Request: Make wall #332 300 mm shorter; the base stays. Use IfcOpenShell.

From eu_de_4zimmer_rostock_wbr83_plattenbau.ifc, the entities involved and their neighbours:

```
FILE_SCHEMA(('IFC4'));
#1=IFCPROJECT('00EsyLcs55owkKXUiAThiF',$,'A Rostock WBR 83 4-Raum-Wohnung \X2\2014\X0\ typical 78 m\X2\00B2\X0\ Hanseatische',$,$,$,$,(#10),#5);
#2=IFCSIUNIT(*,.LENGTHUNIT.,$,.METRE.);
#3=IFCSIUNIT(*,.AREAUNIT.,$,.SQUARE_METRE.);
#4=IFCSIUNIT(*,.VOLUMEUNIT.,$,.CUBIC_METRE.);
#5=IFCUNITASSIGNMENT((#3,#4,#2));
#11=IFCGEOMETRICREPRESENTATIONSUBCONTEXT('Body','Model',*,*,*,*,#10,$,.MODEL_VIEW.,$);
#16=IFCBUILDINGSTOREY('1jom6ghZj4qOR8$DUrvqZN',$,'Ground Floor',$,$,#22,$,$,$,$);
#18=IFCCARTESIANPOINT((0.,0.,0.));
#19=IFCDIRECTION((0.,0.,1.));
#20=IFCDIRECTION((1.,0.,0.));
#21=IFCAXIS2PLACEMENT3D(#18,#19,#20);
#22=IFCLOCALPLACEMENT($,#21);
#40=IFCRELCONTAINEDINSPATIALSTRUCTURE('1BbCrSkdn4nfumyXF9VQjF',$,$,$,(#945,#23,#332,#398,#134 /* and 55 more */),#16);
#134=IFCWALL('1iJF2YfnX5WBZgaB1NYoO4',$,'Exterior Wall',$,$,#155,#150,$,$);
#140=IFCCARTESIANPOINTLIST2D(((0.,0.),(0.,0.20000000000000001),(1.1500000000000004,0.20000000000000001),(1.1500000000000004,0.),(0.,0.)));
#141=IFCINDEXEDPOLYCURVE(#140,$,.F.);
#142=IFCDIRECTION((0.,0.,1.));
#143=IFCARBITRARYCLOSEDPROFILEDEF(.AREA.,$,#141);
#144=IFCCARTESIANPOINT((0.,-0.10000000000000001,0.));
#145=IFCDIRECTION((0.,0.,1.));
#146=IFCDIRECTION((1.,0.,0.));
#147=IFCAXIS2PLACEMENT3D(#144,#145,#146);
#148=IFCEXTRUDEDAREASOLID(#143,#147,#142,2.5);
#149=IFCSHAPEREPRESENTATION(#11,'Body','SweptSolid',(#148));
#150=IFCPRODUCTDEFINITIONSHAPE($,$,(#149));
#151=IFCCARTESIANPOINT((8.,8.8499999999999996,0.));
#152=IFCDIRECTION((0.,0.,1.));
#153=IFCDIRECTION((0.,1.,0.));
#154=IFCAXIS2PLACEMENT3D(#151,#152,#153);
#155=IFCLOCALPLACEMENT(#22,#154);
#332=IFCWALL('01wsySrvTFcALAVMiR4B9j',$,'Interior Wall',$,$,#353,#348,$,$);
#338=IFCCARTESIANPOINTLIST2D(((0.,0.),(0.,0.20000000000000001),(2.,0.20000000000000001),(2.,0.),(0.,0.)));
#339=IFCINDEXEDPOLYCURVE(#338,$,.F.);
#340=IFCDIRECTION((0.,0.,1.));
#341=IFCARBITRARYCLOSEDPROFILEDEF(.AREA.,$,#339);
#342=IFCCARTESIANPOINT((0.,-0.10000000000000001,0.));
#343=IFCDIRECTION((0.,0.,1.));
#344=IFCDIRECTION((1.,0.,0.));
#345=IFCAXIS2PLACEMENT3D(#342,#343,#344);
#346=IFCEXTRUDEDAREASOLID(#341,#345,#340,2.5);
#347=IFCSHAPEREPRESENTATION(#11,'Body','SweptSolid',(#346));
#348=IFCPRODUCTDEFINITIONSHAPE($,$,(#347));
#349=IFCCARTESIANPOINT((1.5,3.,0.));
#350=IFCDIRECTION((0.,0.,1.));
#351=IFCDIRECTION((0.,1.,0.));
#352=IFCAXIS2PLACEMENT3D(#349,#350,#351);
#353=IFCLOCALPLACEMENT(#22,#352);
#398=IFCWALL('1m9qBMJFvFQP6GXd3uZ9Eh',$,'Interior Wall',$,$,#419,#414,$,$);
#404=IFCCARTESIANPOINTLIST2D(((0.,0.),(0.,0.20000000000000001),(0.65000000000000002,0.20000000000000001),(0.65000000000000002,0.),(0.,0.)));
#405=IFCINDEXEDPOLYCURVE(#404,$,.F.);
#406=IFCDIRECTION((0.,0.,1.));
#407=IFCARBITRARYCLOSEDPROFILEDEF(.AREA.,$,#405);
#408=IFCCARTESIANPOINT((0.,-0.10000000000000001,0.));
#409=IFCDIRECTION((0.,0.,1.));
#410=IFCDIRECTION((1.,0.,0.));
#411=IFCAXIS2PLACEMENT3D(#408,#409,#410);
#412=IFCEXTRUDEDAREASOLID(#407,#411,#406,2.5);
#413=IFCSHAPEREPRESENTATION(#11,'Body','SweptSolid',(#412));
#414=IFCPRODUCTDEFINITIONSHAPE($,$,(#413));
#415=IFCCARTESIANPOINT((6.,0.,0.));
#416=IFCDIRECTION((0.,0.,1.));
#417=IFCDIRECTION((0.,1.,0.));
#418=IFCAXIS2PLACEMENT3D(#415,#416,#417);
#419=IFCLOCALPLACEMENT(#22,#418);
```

```python
import ifcopenshell
import ifcopenshell.geom
import ifcopenshell.util.representation
import ifcopenshell.util.shape

model = ifcopenshell.open("eu_de_4zimmer_rostock_wbr83_plattenbau.ifc")
settings = ifcopenshell.geom.settings()


def volume(element):
    """Net volume in cubic metres, openings subtracted."""
    shape = ifcopenshell.geom.create_shape(settings, element)
    return ifcopenshell.util.shape.get_volume(shape.geometry)


wall = model.by_guid("01wsySrvTFcALAVMiR4B9j")
before = volume(wall)

body = ifcopenshell.util.representation.get_representation(wall, "Model", "Body")
solid = body.Items[0]
old_height = solid.Depth
solid.Depth -= 0.3
after = volume(wall)

print(f"height {old_height:g} -> {solid.Depth:g}, volume {before:.3f} -> {after:.3f} m3")

model.write("eu_de_4zimmer_rostock_wbr83_plattenbau_edited.ifc")
```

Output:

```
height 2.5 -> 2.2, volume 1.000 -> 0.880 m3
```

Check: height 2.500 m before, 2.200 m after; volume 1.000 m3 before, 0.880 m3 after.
